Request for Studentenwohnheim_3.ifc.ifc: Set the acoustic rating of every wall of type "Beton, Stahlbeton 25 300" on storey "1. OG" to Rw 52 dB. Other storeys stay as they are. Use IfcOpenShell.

First a look at what the model holds.

```python
import ifcopenshell
import ifcopenshell.util.element

model = ifcopenshell.open("Studentenwohnheim_3.ifc.ifc")
print(model.schema)
storey = next(s for s in model.by_type("IfcBuildingStorey") if s.Name == "1. OG")
walls = [e for e in ifcopenshell.util.element.get_decomposition(storey) if e.is_a("IfcWall")]
seen = {}
for e in walls:
    element_type = ifcopenshell.util.element.get_type(e)
    key = (element_type.Name if element_type != e and element_type else None, ifcopenshell.util.element.get_pset(e, "Pset_WallCommon", "AcousticRating"))
    seen[key] = seen.get(key, 0) + 1
for (name, value), count in sorted(seen.items(), key=str):
    print(count, "x", name, "|", value)
```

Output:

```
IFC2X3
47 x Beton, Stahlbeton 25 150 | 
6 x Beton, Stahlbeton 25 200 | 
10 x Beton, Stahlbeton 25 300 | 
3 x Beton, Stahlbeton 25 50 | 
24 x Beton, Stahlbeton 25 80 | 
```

```python
import ifcopenshell
import ifcopenshell.api.pset
import ifcopenshell.util.element

model = ifcopenshell.open("Studentenwohnheim_3.ifc.ifc")

storey = next(s for s in model.by_type("IfcBuildingStorey") if s.Name == "1. OG")
walls = [e for e in ifcopenshell.util.element.get_decomposition(storey) if e.is_a("IfcWall")]

count = 0
for e in walls:
    element_type = ifcopenshell.util.element.get_type(e)
    if element_type in (None, e) or element_type.Name != "Beton, Stahlbeton 25 300":
        continue
    # add_pset returns the element's existing set when there is one.
    pset = ifcopenshell.api.pset.add_pset(model, product=e, name="Pset_WallCommon")
    ifcopenshell.api.pset.edit_pset(model, pset=pset, properties={"AcousticRating": "Rw 52 dB"})
    count += 1

print(count, "walls updated")

model.write("Studentenwohnheim_3.ifc_edited.ifc")
```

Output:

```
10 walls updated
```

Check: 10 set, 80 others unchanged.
